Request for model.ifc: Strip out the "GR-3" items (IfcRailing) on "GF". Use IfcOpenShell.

First a look at what the model holds.

```python
import ifcopenshell
import ifcopenshell.util.element

model = ifcopenshell.open("model.ifc")
print(model.schema)
storey = next(s for s in model.by_type("IfcBuildingStorey") if s.Name == "GF")
railings = [e for e in ifcopenshell.util.element.get_decomposition(storey) if e.is_a("IfcRailing")]
seen = {}
for e in railings:
    element_type = ifcopenshell.util.element.get_type(e)
    name = element_type.Name if element_type not in (None, e) else None
    seen[name] = seen.get(name, 0) + 1
for name, count in sorted(seen.items(), key=str):
    print(count, "x", name)
```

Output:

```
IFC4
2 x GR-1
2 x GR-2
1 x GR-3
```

```python
import ifcopenshell
import ifcopenshell.api.root
import ifcopenshell.util.element

model = ifcopenshell.open("model.ifc")

storey = next(s for s in model.by_type("IfcBuildingStorey") if s.Name == "GF")
railings = [e for e in ifcopenshell.util.element.get_decomposition(storey) if e.is_a("IfcRailing")]
targets = [e for e in railings if (t := ifcopenshell.util.element.get_type(e)) not in (None, e) and t.Name == "GR-3"]

for e in targets:
    ifcopenshell.api.root.remove_product(model, product=e)
print(len(targets), "removed")

model.write("model_updated.ifc")
```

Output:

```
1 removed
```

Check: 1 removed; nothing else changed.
